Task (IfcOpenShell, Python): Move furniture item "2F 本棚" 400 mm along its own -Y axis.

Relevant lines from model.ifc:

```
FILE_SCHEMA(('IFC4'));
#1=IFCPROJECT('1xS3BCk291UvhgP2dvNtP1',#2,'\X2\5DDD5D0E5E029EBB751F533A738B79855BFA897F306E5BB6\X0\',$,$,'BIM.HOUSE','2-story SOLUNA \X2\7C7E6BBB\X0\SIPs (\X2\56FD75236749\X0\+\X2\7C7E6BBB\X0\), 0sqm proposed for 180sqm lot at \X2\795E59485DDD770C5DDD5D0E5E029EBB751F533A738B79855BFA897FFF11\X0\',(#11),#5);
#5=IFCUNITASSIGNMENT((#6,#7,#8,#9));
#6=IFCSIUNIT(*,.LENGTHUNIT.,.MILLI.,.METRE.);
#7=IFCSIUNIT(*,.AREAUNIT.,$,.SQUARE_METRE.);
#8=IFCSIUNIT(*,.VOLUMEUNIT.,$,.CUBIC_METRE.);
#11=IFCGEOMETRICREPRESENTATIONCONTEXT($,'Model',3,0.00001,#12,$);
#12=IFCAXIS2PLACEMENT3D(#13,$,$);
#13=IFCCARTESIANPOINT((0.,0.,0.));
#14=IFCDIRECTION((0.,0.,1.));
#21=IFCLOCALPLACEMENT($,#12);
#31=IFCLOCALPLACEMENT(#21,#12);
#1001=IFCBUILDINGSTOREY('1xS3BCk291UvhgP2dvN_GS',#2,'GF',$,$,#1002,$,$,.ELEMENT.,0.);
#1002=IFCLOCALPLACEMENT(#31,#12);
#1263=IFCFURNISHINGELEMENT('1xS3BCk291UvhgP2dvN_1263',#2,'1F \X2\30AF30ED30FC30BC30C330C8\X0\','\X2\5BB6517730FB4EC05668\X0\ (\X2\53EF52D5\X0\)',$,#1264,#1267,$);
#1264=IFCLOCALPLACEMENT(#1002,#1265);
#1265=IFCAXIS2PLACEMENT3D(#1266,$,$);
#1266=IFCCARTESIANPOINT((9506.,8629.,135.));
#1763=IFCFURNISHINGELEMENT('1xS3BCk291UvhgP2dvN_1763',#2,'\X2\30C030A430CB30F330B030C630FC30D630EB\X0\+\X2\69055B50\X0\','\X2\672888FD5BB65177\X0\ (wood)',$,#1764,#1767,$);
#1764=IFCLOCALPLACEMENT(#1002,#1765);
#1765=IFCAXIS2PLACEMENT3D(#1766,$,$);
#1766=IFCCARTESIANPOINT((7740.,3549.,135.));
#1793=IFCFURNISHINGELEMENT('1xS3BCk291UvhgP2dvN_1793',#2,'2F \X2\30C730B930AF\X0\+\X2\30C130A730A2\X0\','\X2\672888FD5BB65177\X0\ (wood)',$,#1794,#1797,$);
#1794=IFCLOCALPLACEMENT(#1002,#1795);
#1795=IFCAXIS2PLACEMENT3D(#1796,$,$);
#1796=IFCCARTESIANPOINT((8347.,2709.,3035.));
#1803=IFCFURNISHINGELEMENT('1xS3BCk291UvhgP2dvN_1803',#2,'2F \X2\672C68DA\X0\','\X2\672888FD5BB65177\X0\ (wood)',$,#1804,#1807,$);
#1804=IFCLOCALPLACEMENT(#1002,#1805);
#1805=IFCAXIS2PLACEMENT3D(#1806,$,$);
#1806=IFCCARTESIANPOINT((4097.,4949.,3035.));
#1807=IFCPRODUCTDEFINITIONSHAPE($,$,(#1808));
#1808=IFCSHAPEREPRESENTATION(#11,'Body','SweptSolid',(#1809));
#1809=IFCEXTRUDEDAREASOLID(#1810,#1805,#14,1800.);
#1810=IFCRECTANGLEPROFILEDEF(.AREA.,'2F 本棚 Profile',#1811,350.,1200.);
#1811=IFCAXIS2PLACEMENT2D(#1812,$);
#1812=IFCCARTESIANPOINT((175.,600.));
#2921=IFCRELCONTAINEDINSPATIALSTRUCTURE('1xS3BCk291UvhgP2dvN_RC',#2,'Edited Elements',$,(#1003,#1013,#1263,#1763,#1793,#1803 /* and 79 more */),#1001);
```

```python
import ifcopenshell
import ifcopenshell.api.geometry
import ifcopenshell.util.placement
import ifcopenshell.util.unit

model = ifcopenshell.open("model.ifc")
unit_scale = ifcopenshell.util.unit.calculate_unit_scale(model)

item = model.by_guid("1xS3BCk291UvhgP2dvN_1803")
matrix = ifcopenshell.util.placement.get_local_placement(item.ObjectPlacement)
matrix[:3, 3] -= matrix[:3, 1] * 0.4 / unit_scale
ifcopenshell.api.geometry.edit_object_placement(model, product=item, matrix=matrix, is_si=False)

print(ifcopenshell.util.placement.get_local_placement(item.ObjectPlacement).round(3) + 0.0)

model.write("model_edited.ifc")
```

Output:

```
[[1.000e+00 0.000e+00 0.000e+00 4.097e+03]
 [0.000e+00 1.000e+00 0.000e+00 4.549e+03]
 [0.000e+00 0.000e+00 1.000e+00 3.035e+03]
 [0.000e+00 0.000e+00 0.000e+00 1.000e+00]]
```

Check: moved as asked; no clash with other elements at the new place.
